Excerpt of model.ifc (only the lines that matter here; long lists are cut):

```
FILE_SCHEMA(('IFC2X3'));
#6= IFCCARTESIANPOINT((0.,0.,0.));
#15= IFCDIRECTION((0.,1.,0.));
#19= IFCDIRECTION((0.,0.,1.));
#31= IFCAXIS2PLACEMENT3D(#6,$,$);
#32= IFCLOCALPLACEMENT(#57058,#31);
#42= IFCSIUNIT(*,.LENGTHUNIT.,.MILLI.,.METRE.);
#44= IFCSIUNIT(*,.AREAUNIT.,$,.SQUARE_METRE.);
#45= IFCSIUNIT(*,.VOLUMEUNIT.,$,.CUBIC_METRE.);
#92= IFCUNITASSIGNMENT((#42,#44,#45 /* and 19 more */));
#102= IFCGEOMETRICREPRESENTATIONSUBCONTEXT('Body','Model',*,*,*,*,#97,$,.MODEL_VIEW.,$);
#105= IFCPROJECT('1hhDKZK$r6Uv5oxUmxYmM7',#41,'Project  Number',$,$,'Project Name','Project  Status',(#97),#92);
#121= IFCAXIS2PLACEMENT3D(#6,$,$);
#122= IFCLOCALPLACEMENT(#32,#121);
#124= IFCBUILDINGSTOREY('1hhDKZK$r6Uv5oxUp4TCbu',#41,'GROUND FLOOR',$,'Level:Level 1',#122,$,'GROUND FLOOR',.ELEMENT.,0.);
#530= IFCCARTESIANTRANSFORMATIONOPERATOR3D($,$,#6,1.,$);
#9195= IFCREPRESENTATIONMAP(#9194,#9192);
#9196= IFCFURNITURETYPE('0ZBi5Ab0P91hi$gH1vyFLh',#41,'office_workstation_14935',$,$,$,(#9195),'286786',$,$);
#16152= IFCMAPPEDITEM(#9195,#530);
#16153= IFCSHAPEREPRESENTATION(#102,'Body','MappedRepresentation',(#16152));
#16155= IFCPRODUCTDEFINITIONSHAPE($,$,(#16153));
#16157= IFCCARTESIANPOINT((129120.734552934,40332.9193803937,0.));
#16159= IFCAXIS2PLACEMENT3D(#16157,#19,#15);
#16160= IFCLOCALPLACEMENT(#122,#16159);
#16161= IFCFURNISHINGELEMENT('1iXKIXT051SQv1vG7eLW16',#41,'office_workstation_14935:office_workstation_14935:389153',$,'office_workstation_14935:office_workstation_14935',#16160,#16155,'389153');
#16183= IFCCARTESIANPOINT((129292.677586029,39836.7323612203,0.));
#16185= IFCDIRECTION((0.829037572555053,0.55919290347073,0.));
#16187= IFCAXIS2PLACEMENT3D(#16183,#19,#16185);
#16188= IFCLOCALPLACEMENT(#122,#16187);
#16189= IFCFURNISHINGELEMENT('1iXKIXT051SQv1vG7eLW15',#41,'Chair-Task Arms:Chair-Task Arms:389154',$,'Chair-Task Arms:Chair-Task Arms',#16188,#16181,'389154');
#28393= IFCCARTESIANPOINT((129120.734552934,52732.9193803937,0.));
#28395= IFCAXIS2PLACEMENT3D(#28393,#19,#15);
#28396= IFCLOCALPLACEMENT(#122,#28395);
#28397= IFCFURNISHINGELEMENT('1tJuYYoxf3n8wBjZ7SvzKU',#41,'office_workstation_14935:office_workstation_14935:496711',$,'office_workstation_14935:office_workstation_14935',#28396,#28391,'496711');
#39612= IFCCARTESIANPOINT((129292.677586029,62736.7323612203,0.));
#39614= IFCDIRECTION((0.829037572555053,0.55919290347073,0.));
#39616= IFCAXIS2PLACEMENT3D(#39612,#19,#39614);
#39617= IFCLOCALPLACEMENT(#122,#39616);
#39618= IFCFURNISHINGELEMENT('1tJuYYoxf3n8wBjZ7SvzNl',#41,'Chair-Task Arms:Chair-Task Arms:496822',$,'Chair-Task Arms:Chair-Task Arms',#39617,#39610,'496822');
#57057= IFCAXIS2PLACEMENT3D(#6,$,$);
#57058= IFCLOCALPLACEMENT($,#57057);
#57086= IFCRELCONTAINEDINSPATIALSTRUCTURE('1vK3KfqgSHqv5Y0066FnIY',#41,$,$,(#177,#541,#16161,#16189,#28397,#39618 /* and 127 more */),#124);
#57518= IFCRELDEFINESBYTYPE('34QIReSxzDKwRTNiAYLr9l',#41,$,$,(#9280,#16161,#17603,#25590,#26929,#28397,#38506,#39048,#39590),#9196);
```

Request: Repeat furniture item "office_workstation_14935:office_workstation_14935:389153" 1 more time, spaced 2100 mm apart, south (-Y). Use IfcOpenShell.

```python
import numpy as np
import ifcopenshell
import ifcopenshell.api.geometry
import ifcopenshell.api.root
import ifcopenshell.util.element
import ifcopenshell.util.placement

model = ifcopenshell.open("model.ifc")


def reuse_history(source, copy):
    """copy_class also copies each property set's owner history, people and application; keep the originals."""
    for rel in copy.IsDefinedBy:
        if rel.is_a("IfcRelDefinesByProperties") and (history := rel.RelatingPropertyDefinition.OwnerHistory):
            rel.RelatingPropertyDefinition.OwnerHistory = source.OwnerHistory
            ifcopenshell.util.element.remove_deep2(model, history)


source = model.by_guid("1iXKIXT051SQv1vG7eLW16")
base = ifcopenshell.util.placement.get_local_placement(source.ObjectPlacement)
step = np.array([0.0, -1.0, 0.0]) * 2100.0

for i in range(1, 2):
    copy = ifcopenshell.api.root.copy_class(model, product=source)
    copy.Representation = ifcopenshell.util.element.copy_deep(
        model, source.Representation, exclude=["IfcGeometricRepresentationContext", "IfcRepresentationMap"]
    )
    copy.Name = "office_workstation_14935:office_workstation_14935"
    copy.Tag = None
    reuse_history(source, copy)
    matrix = base.copy()
    matrix[:3, 3] += i * step
    print("added at", matrix[:3, 3].round(3) + 0.0)
    ifcopenshell.api.geometry.edit_object_placement(model, product=copy, matrix=matrix, is_si=False)

model.write("model_updated.ifc")
```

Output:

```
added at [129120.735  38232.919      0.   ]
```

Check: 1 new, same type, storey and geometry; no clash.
